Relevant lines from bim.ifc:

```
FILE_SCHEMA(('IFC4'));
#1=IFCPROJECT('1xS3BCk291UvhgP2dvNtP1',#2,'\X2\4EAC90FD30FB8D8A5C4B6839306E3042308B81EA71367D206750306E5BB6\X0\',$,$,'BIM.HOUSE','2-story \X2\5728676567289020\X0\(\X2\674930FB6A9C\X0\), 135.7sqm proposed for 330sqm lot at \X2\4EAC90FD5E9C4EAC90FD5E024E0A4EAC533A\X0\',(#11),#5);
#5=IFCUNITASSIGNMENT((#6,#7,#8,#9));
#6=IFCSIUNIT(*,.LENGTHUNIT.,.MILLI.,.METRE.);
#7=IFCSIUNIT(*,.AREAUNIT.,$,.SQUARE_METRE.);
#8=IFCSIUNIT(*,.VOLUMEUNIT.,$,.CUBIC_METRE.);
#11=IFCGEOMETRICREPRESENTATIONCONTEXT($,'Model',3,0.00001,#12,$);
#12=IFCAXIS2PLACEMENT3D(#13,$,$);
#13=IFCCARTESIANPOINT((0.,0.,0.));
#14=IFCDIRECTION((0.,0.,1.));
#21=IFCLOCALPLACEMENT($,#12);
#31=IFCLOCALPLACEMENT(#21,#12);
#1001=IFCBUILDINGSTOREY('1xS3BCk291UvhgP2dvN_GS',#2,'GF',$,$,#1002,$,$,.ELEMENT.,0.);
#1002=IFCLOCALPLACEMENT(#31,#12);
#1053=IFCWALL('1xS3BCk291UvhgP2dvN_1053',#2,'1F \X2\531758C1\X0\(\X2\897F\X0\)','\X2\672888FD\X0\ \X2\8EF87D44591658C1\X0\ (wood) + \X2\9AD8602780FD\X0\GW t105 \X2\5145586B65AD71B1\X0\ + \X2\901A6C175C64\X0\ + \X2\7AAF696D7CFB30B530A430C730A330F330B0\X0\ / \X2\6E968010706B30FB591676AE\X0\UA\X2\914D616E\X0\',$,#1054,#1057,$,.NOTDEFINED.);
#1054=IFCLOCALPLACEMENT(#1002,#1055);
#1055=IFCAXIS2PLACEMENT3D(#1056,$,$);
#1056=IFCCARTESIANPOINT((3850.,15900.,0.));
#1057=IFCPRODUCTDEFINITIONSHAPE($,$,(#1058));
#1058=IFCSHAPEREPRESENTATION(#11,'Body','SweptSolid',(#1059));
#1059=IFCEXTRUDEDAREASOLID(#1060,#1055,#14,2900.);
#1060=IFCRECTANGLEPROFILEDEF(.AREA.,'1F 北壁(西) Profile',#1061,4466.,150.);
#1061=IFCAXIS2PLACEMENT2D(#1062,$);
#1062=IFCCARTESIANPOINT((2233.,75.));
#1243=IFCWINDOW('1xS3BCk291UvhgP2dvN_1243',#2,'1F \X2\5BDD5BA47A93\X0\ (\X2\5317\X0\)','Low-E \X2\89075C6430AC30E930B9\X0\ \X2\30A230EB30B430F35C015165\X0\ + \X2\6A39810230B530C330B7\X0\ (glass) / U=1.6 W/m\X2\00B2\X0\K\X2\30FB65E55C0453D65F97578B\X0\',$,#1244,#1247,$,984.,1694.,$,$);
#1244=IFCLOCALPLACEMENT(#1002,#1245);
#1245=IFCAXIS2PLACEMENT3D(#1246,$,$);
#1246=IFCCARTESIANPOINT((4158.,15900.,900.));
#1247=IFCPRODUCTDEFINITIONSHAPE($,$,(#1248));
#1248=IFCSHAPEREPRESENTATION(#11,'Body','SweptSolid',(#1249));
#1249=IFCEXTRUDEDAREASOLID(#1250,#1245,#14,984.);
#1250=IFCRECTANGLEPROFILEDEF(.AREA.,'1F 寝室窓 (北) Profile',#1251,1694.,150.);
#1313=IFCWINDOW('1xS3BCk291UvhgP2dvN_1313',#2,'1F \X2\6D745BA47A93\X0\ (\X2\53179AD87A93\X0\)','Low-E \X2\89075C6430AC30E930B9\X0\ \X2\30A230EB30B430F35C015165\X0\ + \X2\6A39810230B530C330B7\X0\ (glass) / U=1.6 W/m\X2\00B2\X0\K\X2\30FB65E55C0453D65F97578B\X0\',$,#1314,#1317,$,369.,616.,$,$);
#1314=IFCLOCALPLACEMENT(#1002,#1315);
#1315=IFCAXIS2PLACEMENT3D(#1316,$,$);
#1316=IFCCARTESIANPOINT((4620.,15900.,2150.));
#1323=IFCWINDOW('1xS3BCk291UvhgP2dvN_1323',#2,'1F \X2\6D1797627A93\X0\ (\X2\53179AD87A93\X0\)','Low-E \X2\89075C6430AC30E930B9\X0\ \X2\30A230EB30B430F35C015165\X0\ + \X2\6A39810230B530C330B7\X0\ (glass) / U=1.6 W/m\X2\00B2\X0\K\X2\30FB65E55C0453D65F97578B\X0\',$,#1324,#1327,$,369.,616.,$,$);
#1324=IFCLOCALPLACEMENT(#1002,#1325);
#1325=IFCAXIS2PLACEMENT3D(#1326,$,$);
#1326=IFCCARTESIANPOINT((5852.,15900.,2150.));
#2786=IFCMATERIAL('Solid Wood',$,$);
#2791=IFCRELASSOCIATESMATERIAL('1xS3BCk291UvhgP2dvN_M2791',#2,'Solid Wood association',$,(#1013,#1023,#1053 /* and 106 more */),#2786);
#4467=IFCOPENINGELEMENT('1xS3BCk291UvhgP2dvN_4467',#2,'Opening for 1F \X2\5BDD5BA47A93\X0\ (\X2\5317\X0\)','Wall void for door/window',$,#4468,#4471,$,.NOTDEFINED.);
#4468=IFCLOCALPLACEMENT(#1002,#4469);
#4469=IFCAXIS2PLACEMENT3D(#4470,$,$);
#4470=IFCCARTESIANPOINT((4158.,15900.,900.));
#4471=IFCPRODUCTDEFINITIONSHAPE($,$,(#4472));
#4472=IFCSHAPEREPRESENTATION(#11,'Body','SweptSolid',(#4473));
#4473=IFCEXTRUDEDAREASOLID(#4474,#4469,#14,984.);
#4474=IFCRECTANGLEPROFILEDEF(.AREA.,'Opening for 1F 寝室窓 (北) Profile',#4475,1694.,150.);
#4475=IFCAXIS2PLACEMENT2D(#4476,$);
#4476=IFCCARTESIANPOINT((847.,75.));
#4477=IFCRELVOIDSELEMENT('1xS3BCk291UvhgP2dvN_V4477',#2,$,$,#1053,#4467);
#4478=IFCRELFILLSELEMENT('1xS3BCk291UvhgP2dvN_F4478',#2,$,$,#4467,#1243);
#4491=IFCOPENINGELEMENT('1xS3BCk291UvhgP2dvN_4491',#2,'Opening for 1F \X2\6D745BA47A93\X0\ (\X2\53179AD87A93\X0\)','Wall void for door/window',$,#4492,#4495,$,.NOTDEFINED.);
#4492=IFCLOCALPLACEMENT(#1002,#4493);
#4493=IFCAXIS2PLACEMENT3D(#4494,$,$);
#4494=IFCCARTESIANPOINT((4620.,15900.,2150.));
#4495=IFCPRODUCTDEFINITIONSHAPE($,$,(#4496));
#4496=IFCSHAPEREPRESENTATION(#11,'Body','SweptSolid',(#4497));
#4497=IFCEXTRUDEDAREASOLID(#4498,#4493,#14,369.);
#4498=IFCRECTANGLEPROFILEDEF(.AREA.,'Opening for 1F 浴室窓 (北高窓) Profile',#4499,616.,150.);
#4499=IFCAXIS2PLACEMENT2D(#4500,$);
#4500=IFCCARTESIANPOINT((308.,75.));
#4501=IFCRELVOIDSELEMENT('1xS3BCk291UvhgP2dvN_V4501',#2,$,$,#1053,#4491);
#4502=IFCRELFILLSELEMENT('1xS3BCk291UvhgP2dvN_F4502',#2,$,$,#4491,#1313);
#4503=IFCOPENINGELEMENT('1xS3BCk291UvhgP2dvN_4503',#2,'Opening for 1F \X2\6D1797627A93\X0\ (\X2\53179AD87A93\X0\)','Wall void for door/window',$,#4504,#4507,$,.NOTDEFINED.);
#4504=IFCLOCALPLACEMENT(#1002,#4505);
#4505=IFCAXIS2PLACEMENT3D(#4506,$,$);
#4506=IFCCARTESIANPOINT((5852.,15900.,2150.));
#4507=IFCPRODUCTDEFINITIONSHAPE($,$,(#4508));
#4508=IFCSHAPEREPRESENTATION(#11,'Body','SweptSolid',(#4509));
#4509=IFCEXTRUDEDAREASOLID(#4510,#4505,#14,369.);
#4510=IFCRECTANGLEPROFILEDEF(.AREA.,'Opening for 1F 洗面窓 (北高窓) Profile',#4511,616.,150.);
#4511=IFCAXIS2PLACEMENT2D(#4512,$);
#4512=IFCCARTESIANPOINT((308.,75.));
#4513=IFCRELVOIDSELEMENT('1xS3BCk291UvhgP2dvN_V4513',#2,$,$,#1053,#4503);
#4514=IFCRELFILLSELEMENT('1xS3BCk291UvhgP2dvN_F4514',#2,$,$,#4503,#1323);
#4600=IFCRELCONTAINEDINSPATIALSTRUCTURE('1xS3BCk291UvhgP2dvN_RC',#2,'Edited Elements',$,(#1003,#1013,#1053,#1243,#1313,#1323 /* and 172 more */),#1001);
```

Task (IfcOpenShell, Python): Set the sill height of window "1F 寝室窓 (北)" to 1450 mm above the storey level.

```python
import numpy as np
import ifcopenshell
import ifcopenshell.api.geometry
import ifcopenshell.geom
import ifcopenshell.util.element
import ifcopenshell.util.placement
import ifcopenshell.util.shape
import ifcopenshell.util.unit

model = ifcopenshell.open("bim.ifc")
unit_scale = ifcopenshell.util.unit.calculate_unit_scale(model)

window = model.by_guid("1xS3BCk291UvhgP2dvN_1243")
opening = window.FillsVoids[0].RelatingOpeningElement
storey = ifcopenshell.util.element.get_container(window, ifc_class="IfcBuildingStorey")
level = ifcopenshell.util.placement.get_local_placement(storey.ObjectPlacement)[2, 3]

# The opening's origin need not be at the sill, so measure its lowest point.
shape = ifcopenshell.geom.create_shape(ifcopenshell.geom.settings(), opening)
bottom = ifcopenshell.util.shape.get_shape_bottom_elevation(shape, shape.geometry) / unit_scale
dz = level + 1.45 / unit_scale - bottom

shift = np.array([0.0, 0.0, dz])
# The window is not placed relative to its opening, so move both.
for product in (opening, window):
    matrix = ifcopenshell.util.placement.get_local_placement(product.ObjectPlacement)
    matrix[:3, 3] += shift
    ifcopenshell.api.geometry.edit_object_placement(model, product=product, matrix=matrix, is_si=False)

print(f"moved by {dz * unit_scale:+.3f} m")

model.write("bim-out.ifc")
```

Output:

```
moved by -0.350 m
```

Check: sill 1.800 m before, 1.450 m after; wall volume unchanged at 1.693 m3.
